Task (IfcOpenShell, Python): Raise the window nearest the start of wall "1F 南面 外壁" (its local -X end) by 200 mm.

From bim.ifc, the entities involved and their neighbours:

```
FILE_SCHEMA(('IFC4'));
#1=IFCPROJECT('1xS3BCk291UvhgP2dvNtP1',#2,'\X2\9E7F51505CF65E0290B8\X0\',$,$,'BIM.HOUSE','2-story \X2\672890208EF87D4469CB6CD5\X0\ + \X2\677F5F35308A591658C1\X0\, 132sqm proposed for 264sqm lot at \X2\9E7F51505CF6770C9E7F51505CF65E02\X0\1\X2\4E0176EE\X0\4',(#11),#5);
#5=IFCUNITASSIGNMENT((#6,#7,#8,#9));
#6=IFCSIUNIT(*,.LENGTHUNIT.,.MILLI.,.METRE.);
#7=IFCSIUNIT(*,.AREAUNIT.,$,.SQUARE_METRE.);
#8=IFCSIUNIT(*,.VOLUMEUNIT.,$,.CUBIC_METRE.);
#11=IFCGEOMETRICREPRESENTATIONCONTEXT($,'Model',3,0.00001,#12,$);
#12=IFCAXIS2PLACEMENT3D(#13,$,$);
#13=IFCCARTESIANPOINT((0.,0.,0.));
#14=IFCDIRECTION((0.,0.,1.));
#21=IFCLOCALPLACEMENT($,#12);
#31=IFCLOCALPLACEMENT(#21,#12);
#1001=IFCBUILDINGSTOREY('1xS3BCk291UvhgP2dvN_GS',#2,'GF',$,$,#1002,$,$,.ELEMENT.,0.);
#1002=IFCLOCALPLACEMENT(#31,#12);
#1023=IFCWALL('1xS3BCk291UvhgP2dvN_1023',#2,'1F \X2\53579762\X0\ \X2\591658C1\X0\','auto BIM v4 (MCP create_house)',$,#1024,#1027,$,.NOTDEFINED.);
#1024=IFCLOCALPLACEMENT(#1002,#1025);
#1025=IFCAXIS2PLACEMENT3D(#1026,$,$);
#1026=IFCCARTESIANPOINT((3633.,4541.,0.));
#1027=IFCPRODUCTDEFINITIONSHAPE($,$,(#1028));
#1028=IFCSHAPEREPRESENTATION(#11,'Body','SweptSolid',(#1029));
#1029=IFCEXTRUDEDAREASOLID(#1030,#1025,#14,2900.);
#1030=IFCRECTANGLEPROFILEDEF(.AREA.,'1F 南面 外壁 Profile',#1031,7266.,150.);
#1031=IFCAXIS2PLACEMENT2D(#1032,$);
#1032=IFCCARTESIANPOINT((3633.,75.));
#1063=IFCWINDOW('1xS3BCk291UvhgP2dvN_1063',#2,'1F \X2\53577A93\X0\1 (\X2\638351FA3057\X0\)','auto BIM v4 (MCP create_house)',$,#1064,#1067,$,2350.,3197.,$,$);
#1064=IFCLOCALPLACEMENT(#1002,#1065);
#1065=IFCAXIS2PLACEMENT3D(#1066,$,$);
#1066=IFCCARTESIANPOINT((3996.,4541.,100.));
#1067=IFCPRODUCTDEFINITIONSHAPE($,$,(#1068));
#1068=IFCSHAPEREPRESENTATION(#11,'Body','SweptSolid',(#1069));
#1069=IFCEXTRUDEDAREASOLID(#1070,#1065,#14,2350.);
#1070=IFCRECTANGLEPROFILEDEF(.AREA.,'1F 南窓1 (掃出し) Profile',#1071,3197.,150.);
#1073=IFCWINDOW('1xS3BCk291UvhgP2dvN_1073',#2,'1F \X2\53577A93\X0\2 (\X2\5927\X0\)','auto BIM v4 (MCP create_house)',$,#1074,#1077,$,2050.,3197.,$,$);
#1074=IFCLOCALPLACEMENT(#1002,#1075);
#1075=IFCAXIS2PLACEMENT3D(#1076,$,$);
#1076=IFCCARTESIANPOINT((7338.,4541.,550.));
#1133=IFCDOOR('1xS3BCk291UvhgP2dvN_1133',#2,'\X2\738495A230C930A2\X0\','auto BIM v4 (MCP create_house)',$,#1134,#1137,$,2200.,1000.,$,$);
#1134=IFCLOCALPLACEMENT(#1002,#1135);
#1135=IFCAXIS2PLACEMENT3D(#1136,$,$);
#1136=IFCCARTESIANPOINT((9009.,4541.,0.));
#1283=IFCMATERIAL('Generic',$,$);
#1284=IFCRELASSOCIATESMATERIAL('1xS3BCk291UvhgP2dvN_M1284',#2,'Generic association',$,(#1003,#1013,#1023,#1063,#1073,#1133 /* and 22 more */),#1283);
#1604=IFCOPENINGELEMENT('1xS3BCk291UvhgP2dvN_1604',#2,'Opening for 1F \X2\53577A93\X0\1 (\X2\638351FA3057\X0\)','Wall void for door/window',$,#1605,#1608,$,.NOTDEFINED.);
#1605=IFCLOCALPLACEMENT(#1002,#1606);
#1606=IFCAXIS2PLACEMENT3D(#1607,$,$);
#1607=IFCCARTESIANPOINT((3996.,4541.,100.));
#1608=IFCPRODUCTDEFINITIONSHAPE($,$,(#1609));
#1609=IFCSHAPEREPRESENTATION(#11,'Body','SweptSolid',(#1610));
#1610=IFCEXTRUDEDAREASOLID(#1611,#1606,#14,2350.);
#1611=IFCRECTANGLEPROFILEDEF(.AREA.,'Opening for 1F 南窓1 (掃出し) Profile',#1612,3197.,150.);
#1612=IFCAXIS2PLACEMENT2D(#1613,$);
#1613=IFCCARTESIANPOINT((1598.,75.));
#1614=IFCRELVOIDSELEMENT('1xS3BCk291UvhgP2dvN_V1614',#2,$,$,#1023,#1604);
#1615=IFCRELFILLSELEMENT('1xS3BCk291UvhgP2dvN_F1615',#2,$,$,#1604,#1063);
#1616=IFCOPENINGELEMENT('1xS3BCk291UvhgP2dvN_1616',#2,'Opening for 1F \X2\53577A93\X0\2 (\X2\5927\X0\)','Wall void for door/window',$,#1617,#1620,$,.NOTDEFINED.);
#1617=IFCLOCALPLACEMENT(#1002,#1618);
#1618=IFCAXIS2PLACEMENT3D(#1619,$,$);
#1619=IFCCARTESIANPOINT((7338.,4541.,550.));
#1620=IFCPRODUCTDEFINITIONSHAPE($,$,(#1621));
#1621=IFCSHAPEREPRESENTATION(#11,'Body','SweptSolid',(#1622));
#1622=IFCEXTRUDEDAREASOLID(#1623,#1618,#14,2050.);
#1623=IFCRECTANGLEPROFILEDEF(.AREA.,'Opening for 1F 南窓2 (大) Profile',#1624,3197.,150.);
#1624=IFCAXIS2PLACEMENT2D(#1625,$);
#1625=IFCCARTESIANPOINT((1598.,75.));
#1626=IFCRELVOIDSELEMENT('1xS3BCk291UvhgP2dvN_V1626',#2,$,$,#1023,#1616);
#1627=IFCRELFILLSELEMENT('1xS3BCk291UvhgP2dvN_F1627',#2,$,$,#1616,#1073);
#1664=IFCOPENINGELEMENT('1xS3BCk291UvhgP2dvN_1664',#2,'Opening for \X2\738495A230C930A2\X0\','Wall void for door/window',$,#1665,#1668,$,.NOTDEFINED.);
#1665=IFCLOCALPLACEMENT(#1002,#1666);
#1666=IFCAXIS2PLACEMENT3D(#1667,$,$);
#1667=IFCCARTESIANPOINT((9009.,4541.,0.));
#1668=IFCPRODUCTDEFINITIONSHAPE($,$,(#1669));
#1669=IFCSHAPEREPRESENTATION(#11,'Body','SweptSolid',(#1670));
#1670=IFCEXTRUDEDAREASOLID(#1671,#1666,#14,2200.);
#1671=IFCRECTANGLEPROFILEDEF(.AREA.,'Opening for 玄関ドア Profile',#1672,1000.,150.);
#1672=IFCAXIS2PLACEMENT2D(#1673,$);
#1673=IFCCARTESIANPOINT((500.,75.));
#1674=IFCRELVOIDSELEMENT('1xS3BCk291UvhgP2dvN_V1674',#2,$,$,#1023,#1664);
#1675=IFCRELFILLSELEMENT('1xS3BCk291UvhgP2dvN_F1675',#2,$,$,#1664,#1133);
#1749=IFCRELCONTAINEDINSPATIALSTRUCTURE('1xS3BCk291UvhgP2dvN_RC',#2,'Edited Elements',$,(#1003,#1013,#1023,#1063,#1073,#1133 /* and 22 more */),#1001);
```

```python
import numpy as np
import ifcopenshell
import ifcopenshell.api.geometry
import ifcopenshell.util.placement
import ifcopenshell.util.unit

model = ifcopenshell.open("bim.ifc")
unit_scale = ifcopenshell.util.unit.calculate_unit_scale(model)

window = model.by_guid("1xS3BCk291UvhgP2dvN_1063")
opening = window.FillsVoids[0].RelatingOpeningElement
dz = 200.0

shift = np.array([0.0, 0.0, dz])
# The window is not placed relative to its opening, so move both.
for product in (opening, window):
    matrix = ifcopenshell.util.placement.get_local_placement(product.ObjectPlacement)
    matrix[:3, 3] += shift
    ifcopenshell.api.geometry.edit_object_placement(model, product=product, matrix=matrix, is_si=False)

print(f"moved by {dz * unit_scale:+.3f} m")

model.write("bim_v2.ifc")
```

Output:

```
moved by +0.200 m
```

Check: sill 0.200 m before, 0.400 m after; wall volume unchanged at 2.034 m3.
